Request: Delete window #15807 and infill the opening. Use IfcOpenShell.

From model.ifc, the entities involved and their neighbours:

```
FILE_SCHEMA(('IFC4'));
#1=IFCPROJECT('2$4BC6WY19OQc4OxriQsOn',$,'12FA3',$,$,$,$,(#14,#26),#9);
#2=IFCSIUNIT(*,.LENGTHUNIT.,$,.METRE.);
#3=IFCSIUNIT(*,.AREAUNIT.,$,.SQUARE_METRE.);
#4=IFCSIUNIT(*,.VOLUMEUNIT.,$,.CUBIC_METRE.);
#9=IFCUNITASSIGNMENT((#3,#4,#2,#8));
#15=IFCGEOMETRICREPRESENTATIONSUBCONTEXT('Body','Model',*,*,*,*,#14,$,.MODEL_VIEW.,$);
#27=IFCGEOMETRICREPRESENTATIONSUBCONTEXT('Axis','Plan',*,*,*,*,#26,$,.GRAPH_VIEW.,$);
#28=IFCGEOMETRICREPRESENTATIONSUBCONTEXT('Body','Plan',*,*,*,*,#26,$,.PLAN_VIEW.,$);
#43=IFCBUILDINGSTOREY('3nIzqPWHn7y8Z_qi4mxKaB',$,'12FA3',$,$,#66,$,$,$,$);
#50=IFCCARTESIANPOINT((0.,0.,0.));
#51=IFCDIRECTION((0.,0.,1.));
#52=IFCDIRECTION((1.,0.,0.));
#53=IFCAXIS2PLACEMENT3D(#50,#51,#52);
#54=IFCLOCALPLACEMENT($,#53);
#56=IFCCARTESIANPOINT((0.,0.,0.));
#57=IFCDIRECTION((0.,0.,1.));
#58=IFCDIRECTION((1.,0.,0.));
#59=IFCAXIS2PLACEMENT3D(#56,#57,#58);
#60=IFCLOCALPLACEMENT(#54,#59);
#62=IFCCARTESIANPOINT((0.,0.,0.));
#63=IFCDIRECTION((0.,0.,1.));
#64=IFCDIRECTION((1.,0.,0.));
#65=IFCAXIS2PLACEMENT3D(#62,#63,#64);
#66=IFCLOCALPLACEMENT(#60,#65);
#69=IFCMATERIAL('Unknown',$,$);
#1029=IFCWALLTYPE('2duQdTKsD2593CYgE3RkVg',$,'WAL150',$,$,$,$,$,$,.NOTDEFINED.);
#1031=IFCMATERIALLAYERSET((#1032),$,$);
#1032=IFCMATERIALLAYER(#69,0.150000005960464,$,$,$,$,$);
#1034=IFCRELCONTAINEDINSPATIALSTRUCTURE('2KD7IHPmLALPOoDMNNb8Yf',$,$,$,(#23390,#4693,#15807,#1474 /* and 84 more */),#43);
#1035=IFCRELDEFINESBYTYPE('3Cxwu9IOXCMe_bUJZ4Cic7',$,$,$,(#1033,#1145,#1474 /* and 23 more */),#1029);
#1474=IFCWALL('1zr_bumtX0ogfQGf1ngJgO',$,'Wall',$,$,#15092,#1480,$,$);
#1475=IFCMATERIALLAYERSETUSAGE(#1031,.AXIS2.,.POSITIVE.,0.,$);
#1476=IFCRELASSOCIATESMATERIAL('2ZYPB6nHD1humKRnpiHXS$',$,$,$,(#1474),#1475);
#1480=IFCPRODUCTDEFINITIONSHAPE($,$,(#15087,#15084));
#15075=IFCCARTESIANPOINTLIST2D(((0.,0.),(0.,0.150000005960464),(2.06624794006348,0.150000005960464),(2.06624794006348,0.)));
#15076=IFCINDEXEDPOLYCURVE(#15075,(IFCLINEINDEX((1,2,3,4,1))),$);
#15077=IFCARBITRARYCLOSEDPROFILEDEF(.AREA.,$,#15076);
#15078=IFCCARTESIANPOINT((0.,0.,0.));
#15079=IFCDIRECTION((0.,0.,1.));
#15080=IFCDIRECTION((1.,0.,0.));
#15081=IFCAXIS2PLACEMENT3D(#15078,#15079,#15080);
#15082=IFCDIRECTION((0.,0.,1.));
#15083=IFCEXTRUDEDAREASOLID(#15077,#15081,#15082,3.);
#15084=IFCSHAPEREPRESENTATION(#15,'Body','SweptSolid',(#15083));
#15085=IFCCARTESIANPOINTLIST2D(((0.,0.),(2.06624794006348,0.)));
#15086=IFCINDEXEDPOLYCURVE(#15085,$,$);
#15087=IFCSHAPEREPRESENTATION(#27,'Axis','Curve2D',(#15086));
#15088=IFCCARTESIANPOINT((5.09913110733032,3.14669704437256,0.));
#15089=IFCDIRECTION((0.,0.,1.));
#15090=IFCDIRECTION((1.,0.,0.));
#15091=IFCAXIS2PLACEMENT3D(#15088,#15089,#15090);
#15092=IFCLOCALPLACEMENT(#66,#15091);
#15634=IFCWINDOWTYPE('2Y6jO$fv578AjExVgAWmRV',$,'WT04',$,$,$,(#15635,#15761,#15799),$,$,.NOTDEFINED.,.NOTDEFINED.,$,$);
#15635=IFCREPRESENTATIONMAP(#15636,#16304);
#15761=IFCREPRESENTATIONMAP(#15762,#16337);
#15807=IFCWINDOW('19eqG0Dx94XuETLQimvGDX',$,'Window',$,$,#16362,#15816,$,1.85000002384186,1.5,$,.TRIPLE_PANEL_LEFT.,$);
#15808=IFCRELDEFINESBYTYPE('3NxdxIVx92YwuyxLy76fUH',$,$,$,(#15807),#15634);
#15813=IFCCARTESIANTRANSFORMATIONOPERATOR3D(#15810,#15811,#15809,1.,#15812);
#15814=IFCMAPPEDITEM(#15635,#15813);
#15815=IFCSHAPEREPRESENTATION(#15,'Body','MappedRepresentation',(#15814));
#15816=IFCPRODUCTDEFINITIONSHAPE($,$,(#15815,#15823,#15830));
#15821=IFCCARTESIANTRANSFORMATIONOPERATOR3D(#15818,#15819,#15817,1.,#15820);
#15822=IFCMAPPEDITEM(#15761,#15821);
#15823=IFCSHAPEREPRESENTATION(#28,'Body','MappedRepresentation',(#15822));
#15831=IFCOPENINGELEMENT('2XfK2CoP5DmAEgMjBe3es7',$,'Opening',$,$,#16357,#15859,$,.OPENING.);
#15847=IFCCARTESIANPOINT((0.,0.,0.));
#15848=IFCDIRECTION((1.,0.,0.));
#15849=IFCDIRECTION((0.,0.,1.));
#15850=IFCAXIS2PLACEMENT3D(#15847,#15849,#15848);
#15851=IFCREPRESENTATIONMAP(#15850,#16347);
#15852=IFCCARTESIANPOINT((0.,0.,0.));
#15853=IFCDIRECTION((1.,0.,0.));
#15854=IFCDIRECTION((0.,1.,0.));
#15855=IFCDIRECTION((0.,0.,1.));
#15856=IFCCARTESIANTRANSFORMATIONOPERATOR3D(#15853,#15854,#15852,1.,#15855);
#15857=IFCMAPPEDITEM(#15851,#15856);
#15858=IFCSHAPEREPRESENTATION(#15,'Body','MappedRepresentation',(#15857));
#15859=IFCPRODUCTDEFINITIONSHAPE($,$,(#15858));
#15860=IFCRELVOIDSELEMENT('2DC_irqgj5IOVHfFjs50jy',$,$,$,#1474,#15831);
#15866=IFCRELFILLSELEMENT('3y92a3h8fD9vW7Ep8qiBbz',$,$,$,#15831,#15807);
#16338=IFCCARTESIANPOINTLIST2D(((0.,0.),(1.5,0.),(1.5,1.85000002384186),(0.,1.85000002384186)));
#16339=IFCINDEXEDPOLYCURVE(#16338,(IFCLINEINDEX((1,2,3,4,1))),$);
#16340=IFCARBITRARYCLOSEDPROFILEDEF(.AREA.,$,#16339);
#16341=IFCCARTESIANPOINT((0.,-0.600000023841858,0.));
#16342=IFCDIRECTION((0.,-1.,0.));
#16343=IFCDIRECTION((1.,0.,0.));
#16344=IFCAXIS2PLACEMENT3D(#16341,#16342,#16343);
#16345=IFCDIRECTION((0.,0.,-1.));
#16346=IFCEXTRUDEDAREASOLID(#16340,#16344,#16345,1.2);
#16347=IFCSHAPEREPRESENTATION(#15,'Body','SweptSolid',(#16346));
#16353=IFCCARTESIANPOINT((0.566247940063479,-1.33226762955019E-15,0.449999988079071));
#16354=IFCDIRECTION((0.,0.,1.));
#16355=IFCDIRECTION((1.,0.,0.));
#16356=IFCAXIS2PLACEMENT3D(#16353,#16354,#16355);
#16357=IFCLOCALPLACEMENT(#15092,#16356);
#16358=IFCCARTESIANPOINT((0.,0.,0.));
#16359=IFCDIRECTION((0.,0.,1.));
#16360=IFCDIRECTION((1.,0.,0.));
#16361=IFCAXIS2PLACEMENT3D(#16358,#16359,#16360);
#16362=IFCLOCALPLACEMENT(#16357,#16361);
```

```python
import ifcopenshell
import ifcopenshell.api.feature
import ifcopenshell.api.root
import ifcopenshell.geom
import ifcopenshell.util.shape

model = ifcopenshell.open("model.ifc")
settings = ifcopenshell.geom.settings()


def volume(element):
    """Net volume in cubic metres, openings subtracted."""
    shape = ifcopenshell.geom.create_shape(settings, element)
    return ifcopenshell.util.shape.get_volume(shape.geometry)


window = model.by_guid("19eqG0Dx94XuETLQimvGDX")
opening = window.FillsVoids[0].RelatingOpeningElement
wall = opening.VoidsElements[0].RelatingBuildingElement
before = volume(wall)

ifcopenshell.api.root.remove_product(model, product=window)
ifcopenshell.api.feature.remove_feature(model, feature=opening)

after = volume(wall)

print(f"wall volume {before:.3f} -> {after:.3f} m3")

model.write("model_rev.ifc")
```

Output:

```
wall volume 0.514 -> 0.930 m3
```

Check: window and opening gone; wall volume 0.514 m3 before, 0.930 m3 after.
